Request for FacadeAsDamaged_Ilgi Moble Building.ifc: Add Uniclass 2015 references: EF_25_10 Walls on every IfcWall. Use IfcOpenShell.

First a look at what the model holds.

```python
import ifcopenshell

model = ifcopenshell.open("FacadeAsDamaged_Ilgi Moble Building.ifc")
print(model.schema)
print("classifications:", [c.Name for c in model.by_type("IfcClassification")])
for ifc_class in ("IfcDoor", "IfcRoof", "IfcStair", "IfcWall", "IfcWindow"):
    print(ifc_class, len(model.by_type(ifc_class)))
```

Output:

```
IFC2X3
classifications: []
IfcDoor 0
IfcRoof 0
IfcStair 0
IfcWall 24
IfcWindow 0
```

```python
import ifcopenshell
import ifcopenshell.api.classification

model = ifcopenshell.open("FacadeAsDamaged_Ilgi Moble Building.ifc")

# IFC2X3 requires Source and Edition and has no link from the project to the system.
system = model.create_entity("IfcClassification", Source="NBS", Edition="2015", Name="Uniclass 2015")

codes = {
    "IfcWall": ("EF_25_10", "Walls"),
}
for ifc_class, (code, name) in codes.items():
    products = model.by_type(ifc_class)
    ifcopenshell.api.classification.add_reference(
        model, products=products, classification=system, identification=code, name=name
    )
    print(code, len(products))

model.write("FacadeAsDamaged_Ilgi Moble Building_edited.ifc")
```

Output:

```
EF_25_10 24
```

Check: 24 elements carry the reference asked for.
